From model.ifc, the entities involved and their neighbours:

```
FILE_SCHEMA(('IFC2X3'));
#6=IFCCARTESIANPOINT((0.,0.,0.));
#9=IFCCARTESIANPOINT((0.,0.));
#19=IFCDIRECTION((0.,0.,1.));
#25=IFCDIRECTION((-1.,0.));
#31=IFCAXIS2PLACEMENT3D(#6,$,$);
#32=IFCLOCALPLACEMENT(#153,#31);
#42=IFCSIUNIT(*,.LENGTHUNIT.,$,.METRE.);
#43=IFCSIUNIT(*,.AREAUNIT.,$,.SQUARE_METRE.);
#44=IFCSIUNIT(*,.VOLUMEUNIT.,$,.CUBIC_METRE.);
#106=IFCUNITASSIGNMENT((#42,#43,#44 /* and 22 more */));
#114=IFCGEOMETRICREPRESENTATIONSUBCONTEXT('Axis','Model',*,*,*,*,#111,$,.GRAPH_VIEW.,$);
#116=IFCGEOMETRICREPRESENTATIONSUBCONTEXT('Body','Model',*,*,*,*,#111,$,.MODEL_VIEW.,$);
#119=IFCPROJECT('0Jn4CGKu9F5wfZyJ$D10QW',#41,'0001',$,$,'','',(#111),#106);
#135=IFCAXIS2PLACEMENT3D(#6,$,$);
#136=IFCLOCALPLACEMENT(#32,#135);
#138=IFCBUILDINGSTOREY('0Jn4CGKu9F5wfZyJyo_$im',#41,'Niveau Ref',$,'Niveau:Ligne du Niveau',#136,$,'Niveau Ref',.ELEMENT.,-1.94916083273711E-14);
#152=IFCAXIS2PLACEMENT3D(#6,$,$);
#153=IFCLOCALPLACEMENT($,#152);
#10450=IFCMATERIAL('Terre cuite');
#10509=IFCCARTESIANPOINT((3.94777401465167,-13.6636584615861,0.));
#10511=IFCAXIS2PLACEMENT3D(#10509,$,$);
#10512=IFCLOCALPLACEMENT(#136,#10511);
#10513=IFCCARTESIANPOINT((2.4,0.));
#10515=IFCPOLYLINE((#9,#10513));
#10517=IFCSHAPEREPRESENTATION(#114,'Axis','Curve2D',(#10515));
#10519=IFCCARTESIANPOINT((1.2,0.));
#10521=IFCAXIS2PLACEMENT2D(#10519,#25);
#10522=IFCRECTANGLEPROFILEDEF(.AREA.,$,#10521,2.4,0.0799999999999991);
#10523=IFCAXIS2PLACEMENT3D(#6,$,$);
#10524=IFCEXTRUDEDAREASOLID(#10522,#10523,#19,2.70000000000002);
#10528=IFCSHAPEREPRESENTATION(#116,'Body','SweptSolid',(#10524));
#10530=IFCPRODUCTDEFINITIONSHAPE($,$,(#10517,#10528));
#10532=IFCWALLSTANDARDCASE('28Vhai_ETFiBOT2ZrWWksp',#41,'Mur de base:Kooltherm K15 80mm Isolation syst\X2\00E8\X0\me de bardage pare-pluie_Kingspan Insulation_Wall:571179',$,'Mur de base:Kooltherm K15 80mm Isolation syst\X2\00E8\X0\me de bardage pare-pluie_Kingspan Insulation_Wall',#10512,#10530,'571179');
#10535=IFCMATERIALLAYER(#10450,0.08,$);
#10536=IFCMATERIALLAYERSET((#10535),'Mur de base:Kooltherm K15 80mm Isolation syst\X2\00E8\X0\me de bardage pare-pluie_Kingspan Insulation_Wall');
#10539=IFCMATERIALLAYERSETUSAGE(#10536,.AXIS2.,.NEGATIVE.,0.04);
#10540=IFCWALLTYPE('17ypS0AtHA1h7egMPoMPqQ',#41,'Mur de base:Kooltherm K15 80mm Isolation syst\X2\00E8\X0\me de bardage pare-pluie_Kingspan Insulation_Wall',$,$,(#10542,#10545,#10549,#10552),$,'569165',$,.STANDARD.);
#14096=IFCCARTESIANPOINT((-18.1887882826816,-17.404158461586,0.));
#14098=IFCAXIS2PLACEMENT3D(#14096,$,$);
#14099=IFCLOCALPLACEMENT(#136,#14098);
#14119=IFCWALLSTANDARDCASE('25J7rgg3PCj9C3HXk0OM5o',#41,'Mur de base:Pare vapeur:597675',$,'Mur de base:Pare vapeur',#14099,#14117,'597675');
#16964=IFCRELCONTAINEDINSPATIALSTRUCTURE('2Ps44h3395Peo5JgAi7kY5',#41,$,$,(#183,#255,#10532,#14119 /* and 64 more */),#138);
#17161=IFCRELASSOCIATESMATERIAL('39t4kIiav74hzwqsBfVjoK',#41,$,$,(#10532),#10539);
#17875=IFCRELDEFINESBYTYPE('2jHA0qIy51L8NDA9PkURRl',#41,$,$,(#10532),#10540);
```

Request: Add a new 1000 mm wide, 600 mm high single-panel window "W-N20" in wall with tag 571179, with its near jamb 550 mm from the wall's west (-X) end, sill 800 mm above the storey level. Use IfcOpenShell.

```python
import numpy as np
import ifcopenshell
import ifcopenshell.api.feature
import ifcopenshell.api.geometry
import ifcopenshell.api.root
import ifcopenshell.api.spatial
import ifcopenshell.api.type
import ifcopenshell.geom
import ifcopenshell.util.element
import ifcopenshell.util.placement
import ifcopenshell.util.representation
import ifcopenshell.util.shape
import ifcopenshell.util.unit

model = ifcopenshell.open("model.ifc")
unit_scale = ifcopenshell.util.unit.calculate_unit_scale(model)
settings = ifcopenshell.geom.settings()


def volume(element):
    """Net volume in cubic metres, openings subtracted."""
    shape = ifcopenshell.geom.create_shape(settings, element)
    return ifcopenshell.util.shape.get_volume(shape.geometry)


wall = model.by_id(10532)
storey = ifcopenshell.util.element.get_container(wall, ifc_class="IfcBuildingStorey")
context = ifcopenshell.util.representation.get_context(model, "Model", "Body", "MODEL_VIEW")
before = volume(wall)

width, height, from_end, sill = 1, 0.6, 0.55, 0.8  # metres

# The wall runs along its own X axis, and the end named is its -X end.
wall_shape = ifcopenshell.geom.create_shape(settings, wall)
x, y, z = ifcopenshell.util.shape.get_vertices(wall_shape.geometry).T
start = x.min() + from_end
face, thickness = float(y.min()), float(y.max() - y.min())
wall_matrix = ifcopenshell.util.placement.get_local_placement(wall.ObjectPlacement)
level = ifcopenshell.util.placement.get_local_placement(storey.ObjectPlacement)[2, 3]


def in_wall(x, y):
    """Placement at x, y metres in the wall's axes, at sill height."""
    matrix = wall_matrix.copy()
    matrix[:, 3] = wall_matrix @ np.array([x / unit_scale, y / unit_scale, 0.0, 1.0])
    matrix[2, 3] = level + sill / unit_scale
    return matrix


# Opening: a box that overshoots both wall faces by 50 mm.
opening = ifcopenshell.api.root.create_entity(model, ifc_class="IfcOpeningElement")
box = ifcopenshell.api.geometry.add_wall_representation(
    model, context=context, length=width, height=height, thickness=thickness + 0.1
)
ifcopenshell.api.geometry.assign_representation(model, product=opening, representation=box)
ifcopenshell.api.geometry.edit_object_placement(model, product=opening, matrix=in_wall(start, face - 0.05), is_si=False)
ifcopenshell.api.feature.add_feature(model, feature=opening, element=wall)

window = ifcopenshell.api.root.create_entity(model, ifc_class="IfcWindow", name="W-N20")
window.OverallWidth, window.OverallHeight = width / unit_scale, height / unit_scale
body = ifcopenshell.api.geometry.add_window_representation(
    model,
    context=context,
    overall_width=window.OverallWidth,
    overall_height=window.OverallHeight,
    partition_type="SINGLE_PANEL",
)
ifcopenshell.api.geometry.assign_representation(model, product=window, representation=body)
ifcopenshell.api.spatial.assign_container(model, products=[window], relating_structure=storey)
fills = ifcopenshell.api.feature.add_filling(model, opening=opening, element=window)
fills.OwnerHistory = window.OwnerHistory  # required in IFC2X3

# IFC2X3 keeps the operation on the window style.
style = ifcopenshell.api.root.create_entity(model, ifc_class="IfcWindowStyle", name="W-N20")
style.OperationType, style.ConstructionType = "SINGLE_PANEL", "NOTDEFINED"
style.ParameterTakesPrecedence = style.Sizeable = False
ifcopenshell.api.type.assign_type(model, related_objects=[window], relating_type=style)

# Centre the window in the wall's thickness.
ifcopenshell.api.geometry.edit_object_placement(model, product=window, matrix=in_wall(start, face), is_si=False)
window_shape = ifcopenshell.geom.create_shape(settings, window)
depth = ifcopenshell.util.shape.get_vertices(window_shape.geometry)[:, 1]
offset = face + thickness / 2 - (depth.min() + depth.max()) / 2
ifcopenshell.api.geometry.edit_object_placement(model, product=window, matrix=in_wall(start, offset), is_si=False)

after = volume(wall)

print(f"wall volume {before:.3f} -> {after:.3f} m3")

model.write("model_edited.ifc")
```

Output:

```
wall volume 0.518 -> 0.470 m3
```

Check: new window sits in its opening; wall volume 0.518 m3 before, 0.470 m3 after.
